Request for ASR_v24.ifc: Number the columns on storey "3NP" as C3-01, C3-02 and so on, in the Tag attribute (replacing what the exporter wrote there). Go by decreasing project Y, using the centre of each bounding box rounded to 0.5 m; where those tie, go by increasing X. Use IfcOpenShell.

First a look at what the model holds.

```python
import ifcopenshell
import ifcopenshell.util.element
import ifcopenshell.util.placement

model = ifcopenshell.open("ASR_v24.ifc")
print(model.schema)
storey = next(s for s in model.by_type("IfcBuildingStorey") if s.Name == "3NP")
columns = [e for e in ifcopenshell.util.element.get_decomposition(storey) if e.is_a("IfcColumn")]
for e in sorted(columns, key=lambda e: e.id()):
    origin = ifcopenshell.util.placement.get_local_placement(e.ObjectPlacement)[:3, 3]
    print(e.id(), e.Tag, e.Name, origin.round(2) + 0.0, sep=" | ")
```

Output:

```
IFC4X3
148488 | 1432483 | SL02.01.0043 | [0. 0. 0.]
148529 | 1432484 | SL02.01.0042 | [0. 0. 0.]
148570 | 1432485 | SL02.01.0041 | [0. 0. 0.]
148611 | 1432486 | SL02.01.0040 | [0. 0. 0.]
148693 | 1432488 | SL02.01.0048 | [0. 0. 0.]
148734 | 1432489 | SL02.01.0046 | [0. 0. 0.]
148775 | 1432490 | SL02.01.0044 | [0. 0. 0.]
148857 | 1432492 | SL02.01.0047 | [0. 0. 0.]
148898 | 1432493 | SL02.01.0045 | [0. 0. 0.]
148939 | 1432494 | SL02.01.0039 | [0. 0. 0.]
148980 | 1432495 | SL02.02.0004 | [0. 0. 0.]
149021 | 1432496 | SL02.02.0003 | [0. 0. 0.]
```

```python
import ifcopenshell
import ifcopenshell.geom
import ifcopenshell.util.element
import ifcopenshell.util.shape

model = ifcopenshell.open("ASR_v24.ifc")
settings = ifcopenshell.geom.settings()
settings.set("use-world-coords", True)


def centre(element):
    shape = ifcopenshell.geom.create_shape(settings, element)
    return ifcopenshell.util.shape.get_bbox_centroid(shape.geometry)


storey = next(s for s in model.by_type("IfcBuildingStorey") if s.Name == "3NP")
columns = [e for e in ifcopenshell.util.element.get_decomposition(storey) if e.is_a("IfcColumn")]

# Insertion points can sit at a corner or the storey origin, so sort by the geometry (in metres).
centres = {e: centre(e) for e in columns}
columns.sort(key=lambda e: (-round(centres[e][1] / 0.5), centres[e][0]))

for i, e in enumerate(columns, start=1):
    number = f"C3-{i:02d}"
    e.Tag = number
    print(e.id(), number)

model.write("ASR_v24_updated.ifc")
```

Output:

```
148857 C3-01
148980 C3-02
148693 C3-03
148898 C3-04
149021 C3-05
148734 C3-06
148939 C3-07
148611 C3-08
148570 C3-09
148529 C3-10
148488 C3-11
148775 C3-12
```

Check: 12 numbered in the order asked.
